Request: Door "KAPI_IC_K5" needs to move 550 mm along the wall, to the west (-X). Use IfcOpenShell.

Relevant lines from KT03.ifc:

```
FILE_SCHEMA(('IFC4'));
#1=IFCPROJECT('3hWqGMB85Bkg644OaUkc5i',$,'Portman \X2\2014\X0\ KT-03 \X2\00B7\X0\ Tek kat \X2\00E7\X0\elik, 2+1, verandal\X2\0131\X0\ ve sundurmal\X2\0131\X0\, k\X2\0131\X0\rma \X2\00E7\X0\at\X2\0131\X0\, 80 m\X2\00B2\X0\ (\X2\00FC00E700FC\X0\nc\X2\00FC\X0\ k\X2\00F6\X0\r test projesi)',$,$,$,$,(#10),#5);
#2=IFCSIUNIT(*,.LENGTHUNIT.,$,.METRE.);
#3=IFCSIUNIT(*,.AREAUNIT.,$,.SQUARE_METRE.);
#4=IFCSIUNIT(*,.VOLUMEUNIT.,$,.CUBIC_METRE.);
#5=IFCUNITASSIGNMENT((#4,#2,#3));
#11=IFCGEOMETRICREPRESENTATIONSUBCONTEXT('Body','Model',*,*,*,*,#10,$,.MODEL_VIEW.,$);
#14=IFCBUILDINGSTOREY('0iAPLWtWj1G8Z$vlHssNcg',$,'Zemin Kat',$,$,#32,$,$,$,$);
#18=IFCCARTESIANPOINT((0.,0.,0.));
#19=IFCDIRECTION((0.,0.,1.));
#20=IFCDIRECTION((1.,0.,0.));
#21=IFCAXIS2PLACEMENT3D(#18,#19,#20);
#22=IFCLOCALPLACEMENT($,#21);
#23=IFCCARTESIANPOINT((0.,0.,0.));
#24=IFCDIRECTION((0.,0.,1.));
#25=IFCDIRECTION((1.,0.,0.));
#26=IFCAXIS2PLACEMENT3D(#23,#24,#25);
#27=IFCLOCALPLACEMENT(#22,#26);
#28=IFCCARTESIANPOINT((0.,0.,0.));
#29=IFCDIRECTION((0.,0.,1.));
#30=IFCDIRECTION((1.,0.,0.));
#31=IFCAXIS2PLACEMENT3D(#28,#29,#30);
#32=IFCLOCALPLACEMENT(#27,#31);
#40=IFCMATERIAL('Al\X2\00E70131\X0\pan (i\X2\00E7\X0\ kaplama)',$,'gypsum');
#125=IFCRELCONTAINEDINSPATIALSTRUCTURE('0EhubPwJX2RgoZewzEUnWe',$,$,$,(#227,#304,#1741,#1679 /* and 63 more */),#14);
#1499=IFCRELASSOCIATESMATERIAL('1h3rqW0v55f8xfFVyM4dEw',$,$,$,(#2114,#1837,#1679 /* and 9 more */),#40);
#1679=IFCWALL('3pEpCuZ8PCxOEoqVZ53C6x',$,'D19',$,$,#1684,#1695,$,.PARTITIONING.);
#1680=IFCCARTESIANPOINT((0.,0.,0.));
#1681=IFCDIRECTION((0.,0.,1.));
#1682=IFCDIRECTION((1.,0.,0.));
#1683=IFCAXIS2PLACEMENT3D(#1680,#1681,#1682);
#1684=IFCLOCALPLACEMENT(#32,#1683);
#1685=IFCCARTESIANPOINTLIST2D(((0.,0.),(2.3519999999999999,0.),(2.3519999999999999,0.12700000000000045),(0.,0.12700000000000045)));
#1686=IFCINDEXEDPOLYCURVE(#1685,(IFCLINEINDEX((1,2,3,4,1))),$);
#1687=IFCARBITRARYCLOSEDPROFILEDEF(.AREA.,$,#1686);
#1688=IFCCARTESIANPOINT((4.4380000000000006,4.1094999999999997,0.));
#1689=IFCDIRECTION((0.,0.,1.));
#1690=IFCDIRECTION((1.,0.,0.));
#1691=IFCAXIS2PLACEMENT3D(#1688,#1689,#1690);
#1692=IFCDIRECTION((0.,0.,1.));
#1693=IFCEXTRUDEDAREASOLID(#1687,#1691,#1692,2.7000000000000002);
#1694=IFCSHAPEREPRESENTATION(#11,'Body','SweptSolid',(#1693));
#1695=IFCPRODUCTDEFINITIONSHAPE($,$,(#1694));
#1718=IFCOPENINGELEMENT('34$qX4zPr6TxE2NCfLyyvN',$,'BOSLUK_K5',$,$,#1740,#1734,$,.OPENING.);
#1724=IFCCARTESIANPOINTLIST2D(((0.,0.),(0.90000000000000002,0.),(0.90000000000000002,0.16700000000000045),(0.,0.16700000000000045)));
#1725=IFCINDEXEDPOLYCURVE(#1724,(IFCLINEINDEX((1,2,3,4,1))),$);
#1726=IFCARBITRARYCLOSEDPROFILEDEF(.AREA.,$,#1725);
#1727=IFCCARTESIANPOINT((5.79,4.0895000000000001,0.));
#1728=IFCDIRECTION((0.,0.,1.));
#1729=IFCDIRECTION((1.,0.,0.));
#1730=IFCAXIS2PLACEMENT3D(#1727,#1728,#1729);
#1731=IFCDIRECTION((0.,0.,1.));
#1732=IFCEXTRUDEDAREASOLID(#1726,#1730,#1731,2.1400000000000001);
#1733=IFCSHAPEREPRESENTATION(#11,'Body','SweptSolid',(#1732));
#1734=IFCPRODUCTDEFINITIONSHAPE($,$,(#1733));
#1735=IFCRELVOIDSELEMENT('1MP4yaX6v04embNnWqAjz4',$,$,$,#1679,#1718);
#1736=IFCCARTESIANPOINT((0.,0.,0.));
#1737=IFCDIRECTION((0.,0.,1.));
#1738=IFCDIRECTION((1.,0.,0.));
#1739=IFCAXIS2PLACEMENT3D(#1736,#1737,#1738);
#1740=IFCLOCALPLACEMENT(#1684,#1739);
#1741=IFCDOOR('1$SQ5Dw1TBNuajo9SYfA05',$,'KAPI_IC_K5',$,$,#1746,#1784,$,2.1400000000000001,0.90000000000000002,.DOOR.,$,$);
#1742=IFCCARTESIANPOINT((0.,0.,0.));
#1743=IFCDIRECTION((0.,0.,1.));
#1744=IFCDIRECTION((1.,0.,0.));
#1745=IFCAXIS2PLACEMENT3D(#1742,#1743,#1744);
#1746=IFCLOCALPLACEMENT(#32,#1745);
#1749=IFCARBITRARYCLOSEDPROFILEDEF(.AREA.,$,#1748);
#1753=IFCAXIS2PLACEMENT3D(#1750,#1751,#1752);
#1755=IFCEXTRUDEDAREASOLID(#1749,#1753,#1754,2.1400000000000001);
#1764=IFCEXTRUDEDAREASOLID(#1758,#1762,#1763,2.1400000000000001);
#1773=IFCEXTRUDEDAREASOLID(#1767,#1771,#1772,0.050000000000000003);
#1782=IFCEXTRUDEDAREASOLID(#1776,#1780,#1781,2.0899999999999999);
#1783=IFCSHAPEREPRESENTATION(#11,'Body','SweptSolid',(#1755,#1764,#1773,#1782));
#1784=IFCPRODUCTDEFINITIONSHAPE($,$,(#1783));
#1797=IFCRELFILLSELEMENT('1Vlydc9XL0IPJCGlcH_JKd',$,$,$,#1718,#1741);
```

```python
import ifcopenshell
import ifcopenshell.api.geometry
import ifcopenshell.util.placement

model = ifcopenshell.open("KT03.ifc")

door = model.by_guid("1$SQ5Dw1TBNuajo9SYfA05")
opening = door.FillsVoids[0].RelatingOpeningElement
wall = opening.VoidsElements[0].RelatingBuildingElement

wall_matrix = ifcopenshell.util.placement.get_local_placement(wall.ObjectPlacement)
shift = wall_matrix[:3, 0] * -0.55
before = ifcopenshell.util.placement.get_local_placement(door.ObjectPlacement)[:3, 3].copy()

# The door is not placed relative to its opening, so move both.
for product in (opening, door):
    matrix = ifcopenshell.util.placement.get_local_placement(product.ObjectPlacement)
    matrix[:3, 3] += shift
    ifcopenshell.api.geometry.edit_object_placement(model, product=product, matrix=matrix, is_si=False)

after = ifcopenshell.util.placement.get_local_placement(door.ObjectPlacement)[:3, 3]
print("door moved by", (after - before).round(3) + 0.0)

model.write("KT03-out.ifc")
```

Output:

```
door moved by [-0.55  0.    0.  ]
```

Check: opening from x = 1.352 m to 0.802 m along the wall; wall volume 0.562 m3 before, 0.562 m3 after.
